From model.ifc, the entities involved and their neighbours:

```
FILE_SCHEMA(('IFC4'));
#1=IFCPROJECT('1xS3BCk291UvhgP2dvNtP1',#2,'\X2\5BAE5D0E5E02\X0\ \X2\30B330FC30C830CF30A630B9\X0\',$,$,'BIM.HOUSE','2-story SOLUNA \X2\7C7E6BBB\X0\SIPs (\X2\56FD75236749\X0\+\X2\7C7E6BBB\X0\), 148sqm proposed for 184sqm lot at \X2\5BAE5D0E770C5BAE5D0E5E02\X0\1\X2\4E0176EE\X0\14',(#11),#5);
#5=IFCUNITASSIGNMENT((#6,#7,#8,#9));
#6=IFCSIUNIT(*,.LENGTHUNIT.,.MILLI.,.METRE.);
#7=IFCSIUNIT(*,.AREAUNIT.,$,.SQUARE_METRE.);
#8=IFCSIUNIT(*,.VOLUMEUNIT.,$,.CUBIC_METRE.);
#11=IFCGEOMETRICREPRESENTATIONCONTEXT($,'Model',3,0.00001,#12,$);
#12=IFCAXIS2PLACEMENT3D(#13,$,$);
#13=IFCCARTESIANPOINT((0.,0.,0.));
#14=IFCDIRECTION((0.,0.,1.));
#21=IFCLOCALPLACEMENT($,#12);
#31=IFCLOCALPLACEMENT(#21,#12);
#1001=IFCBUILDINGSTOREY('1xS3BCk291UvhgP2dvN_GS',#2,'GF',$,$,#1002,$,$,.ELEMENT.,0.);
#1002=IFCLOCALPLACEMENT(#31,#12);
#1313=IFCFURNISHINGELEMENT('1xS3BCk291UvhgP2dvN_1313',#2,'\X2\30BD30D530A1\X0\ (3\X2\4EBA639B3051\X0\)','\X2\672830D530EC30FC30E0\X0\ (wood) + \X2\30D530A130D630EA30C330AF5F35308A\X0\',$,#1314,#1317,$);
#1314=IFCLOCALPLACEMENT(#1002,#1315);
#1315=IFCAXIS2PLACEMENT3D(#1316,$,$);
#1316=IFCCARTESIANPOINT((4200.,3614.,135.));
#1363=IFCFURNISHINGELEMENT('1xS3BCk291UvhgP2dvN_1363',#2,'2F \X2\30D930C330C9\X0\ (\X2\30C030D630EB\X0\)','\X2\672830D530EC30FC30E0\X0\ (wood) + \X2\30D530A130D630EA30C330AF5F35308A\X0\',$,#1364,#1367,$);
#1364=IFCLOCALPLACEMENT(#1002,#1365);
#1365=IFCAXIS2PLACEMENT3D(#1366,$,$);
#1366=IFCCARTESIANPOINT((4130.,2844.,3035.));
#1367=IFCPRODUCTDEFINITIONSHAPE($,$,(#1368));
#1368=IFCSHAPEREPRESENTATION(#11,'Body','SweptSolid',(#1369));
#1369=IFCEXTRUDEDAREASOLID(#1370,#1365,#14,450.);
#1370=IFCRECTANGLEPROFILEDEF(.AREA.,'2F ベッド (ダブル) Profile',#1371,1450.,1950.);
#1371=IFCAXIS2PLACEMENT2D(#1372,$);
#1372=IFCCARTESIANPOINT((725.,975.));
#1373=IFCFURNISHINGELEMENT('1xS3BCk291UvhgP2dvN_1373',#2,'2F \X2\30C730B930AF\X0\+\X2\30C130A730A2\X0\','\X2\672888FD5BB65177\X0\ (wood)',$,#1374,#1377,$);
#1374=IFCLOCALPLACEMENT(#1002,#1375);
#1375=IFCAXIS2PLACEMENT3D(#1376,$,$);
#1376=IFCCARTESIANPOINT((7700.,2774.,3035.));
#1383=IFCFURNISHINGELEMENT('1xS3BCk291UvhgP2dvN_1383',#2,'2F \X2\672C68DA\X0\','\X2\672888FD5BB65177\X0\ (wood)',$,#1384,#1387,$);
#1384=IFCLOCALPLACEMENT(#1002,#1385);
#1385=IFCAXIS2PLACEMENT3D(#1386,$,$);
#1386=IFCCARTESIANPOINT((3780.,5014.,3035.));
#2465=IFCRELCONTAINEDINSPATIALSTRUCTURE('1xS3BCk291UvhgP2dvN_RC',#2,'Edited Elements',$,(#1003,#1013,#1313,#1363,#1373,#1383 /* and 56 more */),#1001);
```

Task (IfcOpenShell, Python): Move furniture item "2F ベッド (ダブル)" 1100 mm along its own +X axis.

```python
import ifcopenshell
import ifcopenshell.api.geometry
import ifcopenshell.util.placement
import ifcopenshell.util.unit

model = ifcopenshell.open("model.ifc")
unit_scale = ifcopenshell.util.unit.calculate_unit_scale(model)

item = model.by_guid("1xS3BCk291UvhgP2dvN_1363")
matrix = ifcopenshell.util.placement.get_local_placement(item.ObjectPlacement)
matrix[:3, 3] += matrix[:3, 0] * 1.1 / unit_scale
ifcopenshell.api.geometry.edit_object_placement(model, product=item, matrix=matrix, is_si=False)

print(ifcopenshell.util.placement.get_local_placement(item.ObjectPlacement).round(3) + 0.0)

model.write("model_rev.ifc")
```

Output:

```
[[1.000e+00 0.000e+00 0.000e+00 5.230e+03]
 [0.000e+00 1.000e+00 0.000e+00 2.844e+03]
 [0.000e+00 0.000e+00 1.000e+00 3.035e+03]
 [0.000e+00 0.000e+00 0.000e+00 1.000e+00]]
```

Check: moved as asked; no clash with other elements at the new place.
